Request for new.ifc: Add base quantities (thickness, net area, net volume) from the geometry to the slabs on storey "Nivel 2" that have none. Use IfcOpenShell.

First a look at what the model holds.

```python
import ifcopenshell
import ifcopenshell.util.element
import ifcopenshell.util.unit

model = ifcopenshell.open("new.ifc")
print(model.schema)
for unit_type in ("LENGTHUNIT", "AREAUNIT", "VOLUMEUNIT"):
    print(unit_type, ifcopenshell.util.unit.calculate_unit_scale(model, unit_type))
storey = next(s for s in model.by_type("IfcBuildingStorey") if s.Name == "Nivel 2")
slabs = [e for e in ifcopenshell.util.element.get_decomposition(storey) if e.is_a("IfcSlab")]
for e in sorted(slabs, key=lambda e: e.id()):
    print(e.id(), e.is_a(), e.Name, list(ifcopenshell.util.element.get_psets(e, qtos_only=True)), sep=" | ")
```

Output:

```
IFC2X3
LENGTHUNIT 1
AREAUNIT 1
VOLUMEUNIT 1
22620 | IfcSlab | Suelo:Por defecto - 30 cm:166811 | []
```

```python
import ifcopenshell
import ifcopenshell.api.pset
import ifcopenshell.geom
import ifcopenshell.util.element
import ifcopenshell.util.shape
import ifcopenshell.util.unit

model = ifcopenshell.open("new.ifc")
unit_scale = ifcopenshell.util.unit.calculate_unit_scale(model)
area_scale = ifcopenshell.util.unit.calculate_unit_scale(model, "AREAUNIT")
volume_scale = ifcopenshell.util.unit.calculate_unit_scale(model, "VOLUMEUNIT")
settings = ifcopenshell.geom.settings()

storey = next(s for s in model.by_type("IfcBuildingStorey") if s.Name == "Nivel 2")
slabs = [e for e in ifcopenshell.util.element.get_decomposition(storey) if e.is_a("IfcSlab")]

for e in sorted(slabs, key=lambda e: e.id()):
    if ifcopenshell.util.element.get_psets(e, qtos_only=True, should_inherit=False):
        continue
    # Geometry comes back in metres, in the element's own axes.
    shape = ifcopenshell.geom.create_shape(settings, e)
    values = {
        "Width": ifcopenshell.util.shape.get_z(shape.geometry) / unit_scale,
        "NetArea": ifcopenshell.util.shape.get_footprint_area(shape.geometry) / area_scale,
        "NetVolume": ifcopenshell.util.shape.get_volume(shape.geometry) / volume_scale,
    }
    qto = ifcopenshell.api.pset.add_qto(model, product=e, name="BaseQuantities")
    ifcopenshell.api.pset.edit_qto(model, qto=qto, properties=values)
    print(e.id(), {k: round(v, 3) for k, v in values.items()})

model.write("new_updated.ifc")
```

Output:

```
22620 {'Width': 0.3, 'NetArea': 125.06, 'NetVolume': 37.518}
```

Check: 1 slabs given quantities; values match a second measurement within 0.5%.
